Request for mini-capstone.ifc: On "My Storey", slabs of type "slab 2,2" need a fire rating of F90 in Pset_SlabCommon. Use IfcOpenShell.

First a look at what the model holds.

```python
import ifcopenshell
import ifcopenshell.util.element

model = ifcopenshell.open("mini-capstone.ifc")
print(model.schema)
storey = next(s for s in model.by_type("IfcBuildingStorey") if s.Name == "My Storey")
slabs = [e for e in ifcopenshell.util.element.get_decomposition(storey) if e.is_a("IfcSlab")]
seen = {}
for e in slabs:
    element_type = ifcopenshell.util.element.get_type(e)
    key = (element_type.Name if element_type != e and element_type else None, ifcopenshell.util.element.get_pset(e, "Pset_SlabCommon", "FireRating"))
    seen[key] = seen.get(key, 0) + 1
for (name, value), count in sorted(seen.items(), key=str):
    print(count, "x", name, "|", value)
```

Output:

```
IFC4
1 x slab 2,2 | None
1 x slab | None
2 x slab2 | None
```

```python
import ifcopenshell
import ifcopenshell.api.pset
import ifcopenshell.util.element

model = ifcopenshell.open("mini-capstone.ifc")

storey = next(s for s in model.by_type("IfcBuildingStorey") if s.Name == "My Storey")
slabs = [e for e in ifcopenshell.util.element.get_decomposition(storey) if e.is_a("IfcSlab")]

count = 0
for e in slabs:
    element_type = ifcopenshell.util.element.get_type(e)
    if element_type in (None, e) or element_type.Name != "slab 2,2":
        continue
    # add_pset returns the element's existing set when there is one.
    pset = ifcopenshell.api.pset.add_pset(model, product=e, name="Pset_SlabCommon")
    ifcopenshell.api.pset.edit_pset(model, pset=pset, properties={"FireRating": "F90"})
    count += 1

print(count, "slabs updated")

model.write("mini-capstone_updated.ifc")
```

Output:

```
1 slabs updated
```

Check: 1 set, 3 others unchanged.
